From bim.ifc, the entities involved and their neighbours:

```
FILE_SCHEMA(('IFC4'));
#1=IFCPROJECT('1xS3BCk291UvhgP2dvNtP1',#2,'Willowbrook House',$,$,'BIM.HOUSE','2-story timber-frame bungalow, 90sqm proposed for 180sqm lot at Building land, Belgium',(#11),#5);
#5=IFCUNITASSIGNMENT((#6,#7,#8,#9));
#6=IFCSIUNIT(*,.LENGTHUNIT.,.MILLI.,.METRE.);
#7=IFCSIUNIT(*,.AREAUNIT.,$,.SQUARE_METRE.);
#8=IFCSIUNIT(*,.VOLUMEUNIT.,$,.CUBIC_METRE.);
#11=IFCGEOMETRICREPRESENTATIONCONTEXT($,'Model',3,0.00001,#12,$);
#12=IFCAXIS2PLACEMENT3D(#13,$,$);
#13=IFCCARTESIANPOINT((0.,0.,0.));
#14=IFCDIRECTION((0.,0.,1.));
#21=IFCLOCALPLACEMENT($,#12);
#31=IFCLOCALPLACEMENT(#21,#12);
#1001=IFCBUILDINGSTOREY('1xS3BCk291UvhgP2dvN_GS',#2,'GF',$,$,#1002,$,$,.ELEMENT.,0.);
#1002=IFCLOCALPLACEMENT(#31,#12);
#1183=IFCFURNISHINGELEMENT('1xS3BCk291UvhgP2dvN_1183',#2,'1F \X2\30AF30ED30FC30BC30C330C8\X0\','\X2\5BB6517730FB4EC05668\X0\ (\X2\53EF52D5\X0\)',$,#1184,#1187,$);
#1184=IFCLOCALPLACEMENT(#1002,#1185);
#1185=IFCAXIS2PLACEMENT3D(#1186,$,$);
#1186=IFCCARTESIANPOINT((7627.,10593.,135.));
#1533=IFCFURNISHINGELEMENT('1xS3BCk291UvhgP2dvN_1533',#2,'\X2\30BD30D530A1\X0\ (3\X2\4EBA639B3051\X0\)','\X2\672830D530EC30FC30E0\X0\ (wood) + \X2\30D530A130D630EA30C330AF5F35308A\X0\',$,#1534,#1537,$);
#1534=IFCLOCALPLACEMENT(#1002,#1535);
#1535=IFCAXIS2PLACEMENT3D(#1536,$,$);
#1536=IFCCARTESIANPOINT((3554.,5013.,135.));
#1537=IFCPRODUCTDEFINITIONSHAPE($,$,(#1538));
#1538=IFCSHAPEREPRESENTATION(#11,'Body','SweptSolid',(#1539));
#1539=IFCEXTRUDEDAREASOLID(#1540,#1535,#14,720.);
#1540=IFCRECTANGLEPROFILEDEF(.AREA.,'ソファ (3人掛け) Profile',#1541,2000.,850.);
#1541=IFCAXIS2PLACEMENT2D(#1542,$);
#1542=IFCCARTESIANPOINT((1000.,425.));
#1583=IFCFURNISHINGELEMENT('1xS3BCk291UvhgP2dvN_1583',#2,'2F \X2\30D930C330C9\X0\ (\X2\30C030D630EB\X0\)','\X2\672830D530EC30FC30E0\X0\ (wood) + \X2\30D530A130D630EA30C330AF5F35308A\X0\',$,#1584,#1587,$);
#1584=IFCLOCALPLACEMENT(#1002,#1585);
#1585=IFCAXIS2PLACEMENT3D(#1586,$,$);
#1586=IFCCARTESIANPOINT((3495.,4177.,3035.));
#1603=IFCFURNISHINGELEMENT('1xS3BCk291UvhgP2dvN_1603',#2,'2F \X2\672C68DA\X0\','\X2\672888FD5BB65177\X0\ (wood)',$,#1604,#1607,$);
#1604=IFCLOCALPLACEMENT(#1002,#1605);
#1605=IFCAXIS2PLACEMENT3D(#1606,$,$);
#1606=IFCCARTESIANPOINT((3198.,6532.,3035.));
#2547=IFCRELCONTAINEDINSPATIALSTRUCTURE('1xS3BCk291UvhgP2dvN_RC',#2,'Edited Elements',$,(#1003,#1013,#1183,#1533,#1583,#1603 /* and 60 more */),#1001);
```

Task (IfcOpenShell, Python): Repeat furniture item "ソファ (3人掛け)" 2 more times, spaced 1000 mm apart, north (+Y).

```python
import numpy as np
import ifcopenshell
import ifcopenshell.api.geometry
import ifcopenshell.api.root
import ifcopenshell.util.element
import ifcopenshell.util.placement

model = ifcopenshell.open("bim.ifc")


def reuse_history(source, copy):
    """copy_class also copies each property set's owner history, people and application; keep the originals."""
    for rel in copy.IsDefinedBy:
        if rel.is_a("IfcRelDefinesByProperties") and (history := rel.RelatingPropertyDefinition.OwnerHistory):
            rel.RelatingPropertyDefinition.OwnerHistory = source.OwnerHistory
            ifcopenshell.util.element.remove_deep2(model, history)


source = model.by_guid("1xS3BCk291UvhgP2dvN_1533")
base = ifcopenshell.util.placement.get_local_placement(source.ObjectPlacement)
step = np.array([0.0, 1.0, 0.0]) * 1000.0

for i in range(1, 3):
    copy = ifcopenshell.api.root.copy_class(model, product=source)
    copy.Representation = ifcopenshell.util.element.copy_deep(
        model, source.Representation, exclude=["IfcGeometricRepresentationContext", "IfcRepresentationMap"]
    )
    reuse_history(source, copy)
    matrix = base.copy()
    matrix[:3, 3] += i * step
    print("added at", matrix[:3, 3].round(3) + 0.0)
    ifcopenshell.api.geometry.edit_object_placement(model, product=copy, matrix=matrix, is_si=False)

model.write("bim-out.ifc")
```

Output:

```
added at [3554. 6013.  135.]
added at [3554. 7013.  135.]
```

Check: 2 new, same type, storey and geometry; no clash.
